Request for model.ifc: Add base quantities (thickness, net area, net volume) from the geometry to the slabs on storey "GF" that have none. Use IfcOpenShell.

First a look at what the model holds.

```python
import ifcopenshell
import ifcopenshell.util.element
import ifcopenshell.util.unit

model = ifcopenshell.open("model.ifc")
print(model.schema)
for unit_type in ("LENGTHUNIT", "AREAUNIT", "VOLUMEUNIT"):
    print(unit_type, ifcopenshell.util.unit.calculate_unit_scale(model, unit_type))
storey = next(s for s in model.by_type("IfcBuildingStorey") if s.Name == "GF")
slabs = [e for e in ifcopenshell.util.element.get_decomposition(storey) if e.is_a("IfcSlab")]
for e in sorted(slabs, key=lambda e: e.id()):
    print(e.id(), e.is_a(), e.Name, list(ifcopenshell.util.element.get_psets(e, qtos_only=True)), sep=" | ")
```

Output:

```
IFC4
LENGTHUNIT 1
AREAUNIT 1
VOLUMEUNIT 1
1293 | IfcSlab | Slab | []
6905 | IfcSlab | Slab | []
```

```python
import ifcopenshell
import ifcopenshell.api.pset
import ifcopenshell.geom
import ifcopenshell.util.element
import ifcopenshell.util.shape
import ifcopenshell.util.unit

model = ifcopenshell.open("model.ifc")
unit_scale = ifcopenshell.util.unit.calculate_unit_scale(model)
area_scale = ifcopenshell.util.unit.calculate_unit_scale(model, "AREAUNIT")
volume_scale = ifcopenshell.util.unit.calculate_unit_scale(model, "VOLUMEUNIT")
settings = ifcopenshell.geom.settings()

storey = next(s for s in model.by_type("IfcBuildingStorey") if s.Name == "GF")
slabs = [e for e in ifcopenshell.util.element.get_decomposition(storey) if e.is_a("IfcSlab")]

for e in sorted(slabs, key=lambda e: e.id()):
    if ifcopenshell.util.element.get_psets(e, qtos_only=True, should_inherit=False):
        continue
    # Geometry comes back in metres, in the element's own axes.
    shape = ifcopenshell.geom.create_shape(settings, e)
    values = {
        "Width": ifcopenshell.util.shape.get_z(shape.geometry) / unit_scale,
        "NetArea": ifcopenshell.util.shape.get_footprint_area(shape.geometry) / area_scale,
        "NetVolume": ifcopenshell.util.shape.get_volume(shape.geometry) / volume_scale,
    }
    qto = ifcopenshell.api.pset.add_qto(model, product=e, name="Qto_SlabBaseQuantities")
    ifcopenshell.api.pset.edit_qto(model, qto=qto, properties=values)
    print(e.id(), {k: round(v, 3) for k, v in values.items()})

model.write("model-out.ifc")
```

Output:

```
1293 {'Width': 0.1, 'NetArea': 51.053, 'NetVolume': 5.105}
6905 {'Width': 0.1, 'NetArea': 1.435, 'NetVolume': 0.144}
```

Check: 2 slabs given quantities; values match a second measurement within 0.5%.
